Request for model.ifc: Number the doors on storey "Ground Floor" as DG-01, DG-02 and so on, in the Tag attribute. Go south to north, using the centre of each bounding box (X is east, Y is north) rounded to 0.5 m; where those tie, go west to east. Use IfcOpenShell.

First a look at what the model holds.

```python
import ifcopenshell
import ifcopenshell.util.element
import ifcopenshell.util.placement

model = ifcopenshell.open("model.ifc")
print(model.schema)
storey = next(s for s in model.by_type("IfcBuildingStorey") if s.Name == "Ground Floor")
doors = [e for e in ifcopenshell.util.element.get_decomposition(storey) if e.is_a("IfcDoor")]
for e in sorted(doors, key=lambda e: e.id()):
    origin = ifcopenshell.util.placement.get_local_placement(e.ObjectPlacement)[:3, 3]
    print(e.id(), e.Tag, e.Name, origin.round(2) + 0.0, sep=" | ")
```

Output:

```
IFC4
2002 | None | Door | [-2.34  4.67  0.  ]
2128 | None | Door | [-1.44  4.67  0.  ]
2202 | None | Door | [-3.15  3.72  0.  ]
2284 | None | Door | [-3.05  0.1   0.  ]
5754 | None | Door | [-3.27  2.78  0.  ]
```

```python
import ifcopenshell
import ifcopenshell.geom
import ifcopenshell.util.element
import ifcopenshell.util.shape

model = ifcopenshell.open("model.ifc")
settings = ifcopenshell.geom.settings()
settings.set("use-world-coords", True)


def centre(element):
    shape = ifcopenshell.geom.create_shape(settings, element)
    return ifcopenshell.util.shape.get_bbox_centroid(shape.geometry)


storey = next(s for s in model.by_type("IfcBuildingStorey") if s.Name == "Ground Floor")
doors = [e for e in ifcopenshell.util.element.get_decomposition(storey) if e.is_a("IfcDoor")]

# Insertion points can sit at a corner or the storey origin, so sort by the geometry (in metres).
centres = {e: centre(e) for e in doors}
doors.sort(key=lambda e: (round(centres[e][1] / 0.5), centres[e][0]))

for i, e in enumerate(doors, start=1):
    number = f"DG-{i:02d}"
    e.Tag = number
    print(e.id(), number)

model.write("model_v2.ifc")
```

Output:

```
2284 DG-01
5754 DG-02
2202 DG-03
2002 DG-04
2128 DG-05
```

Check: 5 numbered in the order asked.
